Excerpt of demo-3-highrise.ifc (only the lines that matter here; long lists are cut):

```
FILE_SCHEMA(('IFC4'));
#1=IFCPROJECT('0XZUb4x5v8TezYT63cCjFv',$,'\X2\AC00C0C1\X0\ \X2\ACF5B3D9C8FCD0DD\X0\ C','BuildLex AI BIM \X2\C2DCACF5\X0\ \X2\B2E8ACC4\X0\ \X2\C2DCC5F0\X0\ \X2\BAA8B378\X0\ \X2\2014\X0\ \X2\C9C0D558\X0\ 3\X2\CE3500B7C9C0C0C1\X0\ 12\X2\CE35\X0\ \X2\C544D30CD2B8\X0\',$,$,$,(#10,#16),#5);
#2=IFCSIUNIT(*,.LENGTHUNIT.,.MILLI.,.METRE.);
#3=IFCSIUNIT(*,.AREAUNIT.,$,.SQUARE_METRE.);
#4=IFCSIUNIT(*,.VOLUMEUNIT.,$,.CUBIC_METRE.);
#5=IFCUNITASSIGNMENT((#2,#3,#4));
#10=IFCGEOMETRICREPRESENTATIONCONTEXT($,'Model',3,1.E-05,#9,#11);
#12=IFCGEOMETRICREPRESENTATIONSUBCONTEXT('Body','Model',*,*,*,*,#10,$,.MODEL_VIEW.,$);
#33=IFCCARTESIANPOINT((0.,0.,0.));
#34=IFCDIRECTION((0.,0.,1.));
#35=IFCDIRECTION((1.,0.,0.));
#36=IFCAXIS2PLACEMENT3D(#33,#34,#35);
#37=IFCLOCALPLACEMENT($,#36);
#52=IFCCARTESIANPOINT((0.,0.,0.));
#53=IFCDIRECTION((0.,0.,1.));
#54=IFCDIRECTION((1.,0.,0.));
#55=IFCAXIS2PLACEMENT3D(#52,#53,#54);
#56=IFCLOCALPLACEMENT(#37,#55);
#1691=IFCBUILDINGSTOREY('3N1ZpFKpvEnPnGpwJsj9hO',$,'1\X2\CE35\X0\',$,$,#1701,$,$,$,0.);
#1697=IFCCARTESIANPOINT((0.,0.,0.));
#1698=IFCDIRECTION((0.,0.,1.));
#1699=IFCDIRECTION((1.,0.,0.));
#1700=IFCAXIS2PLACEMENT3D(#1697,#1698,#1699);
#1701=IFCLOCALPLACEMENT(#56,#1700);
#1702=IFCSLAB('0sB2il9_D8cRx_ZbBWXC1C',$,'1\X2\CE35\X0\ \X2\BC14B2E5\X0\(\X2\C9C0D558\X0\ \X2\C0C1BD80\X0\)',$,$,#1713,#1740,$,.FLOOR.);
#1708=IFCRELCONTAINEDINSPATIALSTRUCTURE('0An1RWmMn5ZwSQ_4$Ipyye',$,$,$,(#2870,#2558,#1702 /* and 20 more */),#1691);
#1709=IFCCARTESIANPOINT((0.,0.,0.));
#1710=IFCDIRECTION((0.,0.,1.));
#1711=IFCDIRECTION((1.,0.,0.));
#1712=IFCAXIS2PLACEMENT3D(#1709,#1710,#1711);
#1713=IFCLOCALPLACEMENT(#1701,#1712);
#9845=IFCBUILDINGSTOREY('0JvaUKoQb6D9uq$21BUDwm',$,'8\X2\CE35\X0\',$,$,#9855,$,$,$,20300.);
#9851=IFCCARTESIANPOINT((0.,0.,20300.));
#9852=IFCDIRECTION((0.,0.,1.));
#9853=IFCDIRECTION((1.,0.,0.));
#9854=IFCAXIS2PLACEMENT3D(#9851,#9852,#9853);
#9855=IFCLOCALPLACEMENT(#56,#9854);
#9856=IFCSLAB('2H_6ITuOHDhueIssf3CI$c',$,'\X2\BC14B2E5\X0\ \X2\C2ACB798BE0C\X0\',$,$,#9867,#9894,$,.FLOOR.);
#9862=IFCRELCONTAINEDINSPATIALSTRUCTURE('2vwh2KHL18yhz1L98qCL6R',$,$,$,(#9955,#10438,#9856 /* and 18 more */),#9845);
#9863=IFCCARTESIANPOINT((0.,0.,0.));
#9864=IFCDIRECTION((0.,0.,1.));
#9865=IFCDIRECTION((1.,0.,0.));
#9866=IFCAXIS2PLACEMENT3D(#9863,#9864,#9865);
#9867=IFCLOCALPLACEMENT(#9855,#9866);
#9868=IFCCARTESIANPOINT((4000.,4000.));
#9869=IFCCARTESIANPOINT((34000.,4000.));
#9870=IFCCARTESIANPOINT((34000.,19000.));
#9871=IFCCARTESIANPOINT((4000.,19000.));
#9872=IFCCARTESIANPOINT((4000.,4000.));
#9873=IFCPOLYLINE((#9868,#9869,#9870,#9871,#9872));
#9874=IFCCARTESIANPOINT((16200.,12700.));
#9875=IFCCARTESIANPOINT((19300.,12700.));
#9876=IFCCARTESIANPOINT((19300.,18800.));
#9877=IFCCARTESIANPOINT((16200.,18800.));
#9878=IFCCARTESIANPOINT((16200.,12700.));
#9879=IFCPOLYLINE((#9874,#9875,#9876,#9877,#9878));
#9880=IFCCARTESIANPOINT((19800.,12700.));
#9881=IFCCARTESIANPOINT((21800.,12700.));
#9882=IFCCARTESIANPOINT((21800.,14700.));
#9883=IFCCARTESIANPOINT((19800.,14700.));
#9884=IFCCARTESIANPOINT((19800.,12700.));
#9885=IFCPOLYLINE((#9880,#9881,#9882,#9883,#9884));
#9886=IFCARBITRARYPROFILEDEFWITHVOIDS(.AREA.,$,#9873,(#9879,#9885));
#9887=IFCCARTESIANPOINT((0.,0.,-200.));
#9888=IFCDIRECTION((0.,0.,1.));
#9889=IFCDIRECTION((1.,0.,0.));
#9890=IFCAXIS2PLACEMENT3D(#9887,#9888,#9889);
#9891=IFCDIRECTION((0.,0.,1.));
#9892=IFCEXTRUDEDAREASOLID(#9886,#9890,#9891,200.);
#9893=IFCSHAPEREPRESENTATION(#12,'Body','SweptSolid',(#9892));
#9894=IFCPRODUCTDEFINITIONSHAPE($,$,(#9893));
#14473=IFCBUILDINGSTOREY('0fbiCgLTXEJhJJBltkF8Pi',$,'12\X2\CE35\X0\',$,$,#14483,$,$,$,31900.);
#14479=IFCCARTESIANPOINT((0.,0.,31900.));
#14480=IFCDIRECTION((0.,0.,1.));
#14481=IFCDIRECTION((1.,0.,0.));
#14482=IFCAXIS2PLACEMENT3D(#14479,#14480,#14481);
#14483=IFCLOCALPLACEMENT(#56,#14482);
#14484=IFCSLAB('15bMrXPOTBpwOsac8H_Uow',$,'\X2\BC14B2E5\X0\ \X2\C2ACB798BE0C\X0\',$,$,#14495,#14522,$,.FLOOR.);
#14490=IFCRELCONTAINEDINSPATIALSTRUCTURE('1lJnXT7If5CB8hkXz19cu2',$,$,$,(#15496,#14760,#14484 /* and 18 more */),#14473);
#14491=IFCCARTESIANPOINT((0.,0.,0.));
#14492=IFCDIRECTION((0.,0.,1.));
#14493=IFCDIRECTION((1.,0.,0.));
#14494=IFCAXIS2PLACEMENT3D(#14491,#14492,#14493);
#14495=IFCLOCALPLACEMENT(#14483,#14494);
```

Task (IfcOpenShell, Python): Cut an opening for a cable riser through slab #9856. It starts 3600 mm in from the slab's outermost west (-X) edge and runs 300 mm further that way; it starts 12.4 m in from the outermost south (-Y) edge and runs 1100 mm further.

```python
import numpy as np
import ifcopenshell
import ifcopenshell.api.feature
import ifcopenshell.api.geometry
import ifcopenshell.api.root
import ifcopenshell.geom
import ifcopenshell.util.placement
import ifcopenshell.util.representation
import ifcopenshell.util.shape
import ifcopenshell.util.unit

model = ifcopenshell.open("demo-3-highrise.ifc")
unit_scale = ifcopenshell.util.unit.calculate_unit_scale(model)
settings = ifcopenshell.geom.settings()


def volume(element):
    """Net volume in cubic metres, openings subtracted."""
    shape = ifcopenshell.geom.create_shape(settings, element)
    return ifcopenshell.util.shape.get_volume(shape.geometry)


slab = model.by_guid("2H_6ITuOHDhueIssf3CI$c")
before = volume(slab)

# Extent in the slab's own axes, in metres. The edges named are its -X and -Y sides.
slab_shape = ifcopenshell.geom.create_shape(settings, slab)
vertices = ifcopenshell.util.shape.get_vertices(slab_shape.geometry)
x_min, y_min, bottom = vertices.min(axis=0)
top = vertices[:, 2].max()

opening = ifcopenshell.api.root.create_entity(model, ifc_class="IfcOpeningElement", name="Cable riser opening", predefined_type="OPENING")
context = ifcopenshell.util.representation.get_context(model, "Model", "Body", "MODEL_VIEW")
width, depth = 0.3, 1.1
outline = [(0.0, 0.0), (width, 0.0), (width, depth), (0.0, depth), (0.0, 0.0)]
# Overshoot both faces by 50 mm so the cut is clean.
shape = ifcopenshell.api.geometry.add_slab_representation(
    model, context=context, depth=top - bottom + 0.1, polyline=outline
)
ifcopenshell.api.geometry.assign_representation(model, product=opening, representation=shape)

matrix = ifcopenshell.util.placement.get_local_placement(slab.ObjectPlacement)
matrix[:, 3] = matrix @ np.append(np.array([x_min + 3.6, y_min + 12.4, bottom - 0.05]) / unit_scale, 1.0)
ifcopenshell.api.geometry.edit_object_placement(model, product=opening, matrix=matrix, is_si=False)
ifcopenshell.api.feature.add_feature(model, feature=opening, element=slab)

after = volume(slab)

print(f"slab volume {before:.3f} -> {after:.3f} m3")

model.write("demo-3-highrise_edited.ifc")
```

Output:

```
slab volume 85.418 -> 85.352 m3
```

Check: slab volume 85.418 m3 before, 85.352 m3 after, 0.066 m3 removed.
